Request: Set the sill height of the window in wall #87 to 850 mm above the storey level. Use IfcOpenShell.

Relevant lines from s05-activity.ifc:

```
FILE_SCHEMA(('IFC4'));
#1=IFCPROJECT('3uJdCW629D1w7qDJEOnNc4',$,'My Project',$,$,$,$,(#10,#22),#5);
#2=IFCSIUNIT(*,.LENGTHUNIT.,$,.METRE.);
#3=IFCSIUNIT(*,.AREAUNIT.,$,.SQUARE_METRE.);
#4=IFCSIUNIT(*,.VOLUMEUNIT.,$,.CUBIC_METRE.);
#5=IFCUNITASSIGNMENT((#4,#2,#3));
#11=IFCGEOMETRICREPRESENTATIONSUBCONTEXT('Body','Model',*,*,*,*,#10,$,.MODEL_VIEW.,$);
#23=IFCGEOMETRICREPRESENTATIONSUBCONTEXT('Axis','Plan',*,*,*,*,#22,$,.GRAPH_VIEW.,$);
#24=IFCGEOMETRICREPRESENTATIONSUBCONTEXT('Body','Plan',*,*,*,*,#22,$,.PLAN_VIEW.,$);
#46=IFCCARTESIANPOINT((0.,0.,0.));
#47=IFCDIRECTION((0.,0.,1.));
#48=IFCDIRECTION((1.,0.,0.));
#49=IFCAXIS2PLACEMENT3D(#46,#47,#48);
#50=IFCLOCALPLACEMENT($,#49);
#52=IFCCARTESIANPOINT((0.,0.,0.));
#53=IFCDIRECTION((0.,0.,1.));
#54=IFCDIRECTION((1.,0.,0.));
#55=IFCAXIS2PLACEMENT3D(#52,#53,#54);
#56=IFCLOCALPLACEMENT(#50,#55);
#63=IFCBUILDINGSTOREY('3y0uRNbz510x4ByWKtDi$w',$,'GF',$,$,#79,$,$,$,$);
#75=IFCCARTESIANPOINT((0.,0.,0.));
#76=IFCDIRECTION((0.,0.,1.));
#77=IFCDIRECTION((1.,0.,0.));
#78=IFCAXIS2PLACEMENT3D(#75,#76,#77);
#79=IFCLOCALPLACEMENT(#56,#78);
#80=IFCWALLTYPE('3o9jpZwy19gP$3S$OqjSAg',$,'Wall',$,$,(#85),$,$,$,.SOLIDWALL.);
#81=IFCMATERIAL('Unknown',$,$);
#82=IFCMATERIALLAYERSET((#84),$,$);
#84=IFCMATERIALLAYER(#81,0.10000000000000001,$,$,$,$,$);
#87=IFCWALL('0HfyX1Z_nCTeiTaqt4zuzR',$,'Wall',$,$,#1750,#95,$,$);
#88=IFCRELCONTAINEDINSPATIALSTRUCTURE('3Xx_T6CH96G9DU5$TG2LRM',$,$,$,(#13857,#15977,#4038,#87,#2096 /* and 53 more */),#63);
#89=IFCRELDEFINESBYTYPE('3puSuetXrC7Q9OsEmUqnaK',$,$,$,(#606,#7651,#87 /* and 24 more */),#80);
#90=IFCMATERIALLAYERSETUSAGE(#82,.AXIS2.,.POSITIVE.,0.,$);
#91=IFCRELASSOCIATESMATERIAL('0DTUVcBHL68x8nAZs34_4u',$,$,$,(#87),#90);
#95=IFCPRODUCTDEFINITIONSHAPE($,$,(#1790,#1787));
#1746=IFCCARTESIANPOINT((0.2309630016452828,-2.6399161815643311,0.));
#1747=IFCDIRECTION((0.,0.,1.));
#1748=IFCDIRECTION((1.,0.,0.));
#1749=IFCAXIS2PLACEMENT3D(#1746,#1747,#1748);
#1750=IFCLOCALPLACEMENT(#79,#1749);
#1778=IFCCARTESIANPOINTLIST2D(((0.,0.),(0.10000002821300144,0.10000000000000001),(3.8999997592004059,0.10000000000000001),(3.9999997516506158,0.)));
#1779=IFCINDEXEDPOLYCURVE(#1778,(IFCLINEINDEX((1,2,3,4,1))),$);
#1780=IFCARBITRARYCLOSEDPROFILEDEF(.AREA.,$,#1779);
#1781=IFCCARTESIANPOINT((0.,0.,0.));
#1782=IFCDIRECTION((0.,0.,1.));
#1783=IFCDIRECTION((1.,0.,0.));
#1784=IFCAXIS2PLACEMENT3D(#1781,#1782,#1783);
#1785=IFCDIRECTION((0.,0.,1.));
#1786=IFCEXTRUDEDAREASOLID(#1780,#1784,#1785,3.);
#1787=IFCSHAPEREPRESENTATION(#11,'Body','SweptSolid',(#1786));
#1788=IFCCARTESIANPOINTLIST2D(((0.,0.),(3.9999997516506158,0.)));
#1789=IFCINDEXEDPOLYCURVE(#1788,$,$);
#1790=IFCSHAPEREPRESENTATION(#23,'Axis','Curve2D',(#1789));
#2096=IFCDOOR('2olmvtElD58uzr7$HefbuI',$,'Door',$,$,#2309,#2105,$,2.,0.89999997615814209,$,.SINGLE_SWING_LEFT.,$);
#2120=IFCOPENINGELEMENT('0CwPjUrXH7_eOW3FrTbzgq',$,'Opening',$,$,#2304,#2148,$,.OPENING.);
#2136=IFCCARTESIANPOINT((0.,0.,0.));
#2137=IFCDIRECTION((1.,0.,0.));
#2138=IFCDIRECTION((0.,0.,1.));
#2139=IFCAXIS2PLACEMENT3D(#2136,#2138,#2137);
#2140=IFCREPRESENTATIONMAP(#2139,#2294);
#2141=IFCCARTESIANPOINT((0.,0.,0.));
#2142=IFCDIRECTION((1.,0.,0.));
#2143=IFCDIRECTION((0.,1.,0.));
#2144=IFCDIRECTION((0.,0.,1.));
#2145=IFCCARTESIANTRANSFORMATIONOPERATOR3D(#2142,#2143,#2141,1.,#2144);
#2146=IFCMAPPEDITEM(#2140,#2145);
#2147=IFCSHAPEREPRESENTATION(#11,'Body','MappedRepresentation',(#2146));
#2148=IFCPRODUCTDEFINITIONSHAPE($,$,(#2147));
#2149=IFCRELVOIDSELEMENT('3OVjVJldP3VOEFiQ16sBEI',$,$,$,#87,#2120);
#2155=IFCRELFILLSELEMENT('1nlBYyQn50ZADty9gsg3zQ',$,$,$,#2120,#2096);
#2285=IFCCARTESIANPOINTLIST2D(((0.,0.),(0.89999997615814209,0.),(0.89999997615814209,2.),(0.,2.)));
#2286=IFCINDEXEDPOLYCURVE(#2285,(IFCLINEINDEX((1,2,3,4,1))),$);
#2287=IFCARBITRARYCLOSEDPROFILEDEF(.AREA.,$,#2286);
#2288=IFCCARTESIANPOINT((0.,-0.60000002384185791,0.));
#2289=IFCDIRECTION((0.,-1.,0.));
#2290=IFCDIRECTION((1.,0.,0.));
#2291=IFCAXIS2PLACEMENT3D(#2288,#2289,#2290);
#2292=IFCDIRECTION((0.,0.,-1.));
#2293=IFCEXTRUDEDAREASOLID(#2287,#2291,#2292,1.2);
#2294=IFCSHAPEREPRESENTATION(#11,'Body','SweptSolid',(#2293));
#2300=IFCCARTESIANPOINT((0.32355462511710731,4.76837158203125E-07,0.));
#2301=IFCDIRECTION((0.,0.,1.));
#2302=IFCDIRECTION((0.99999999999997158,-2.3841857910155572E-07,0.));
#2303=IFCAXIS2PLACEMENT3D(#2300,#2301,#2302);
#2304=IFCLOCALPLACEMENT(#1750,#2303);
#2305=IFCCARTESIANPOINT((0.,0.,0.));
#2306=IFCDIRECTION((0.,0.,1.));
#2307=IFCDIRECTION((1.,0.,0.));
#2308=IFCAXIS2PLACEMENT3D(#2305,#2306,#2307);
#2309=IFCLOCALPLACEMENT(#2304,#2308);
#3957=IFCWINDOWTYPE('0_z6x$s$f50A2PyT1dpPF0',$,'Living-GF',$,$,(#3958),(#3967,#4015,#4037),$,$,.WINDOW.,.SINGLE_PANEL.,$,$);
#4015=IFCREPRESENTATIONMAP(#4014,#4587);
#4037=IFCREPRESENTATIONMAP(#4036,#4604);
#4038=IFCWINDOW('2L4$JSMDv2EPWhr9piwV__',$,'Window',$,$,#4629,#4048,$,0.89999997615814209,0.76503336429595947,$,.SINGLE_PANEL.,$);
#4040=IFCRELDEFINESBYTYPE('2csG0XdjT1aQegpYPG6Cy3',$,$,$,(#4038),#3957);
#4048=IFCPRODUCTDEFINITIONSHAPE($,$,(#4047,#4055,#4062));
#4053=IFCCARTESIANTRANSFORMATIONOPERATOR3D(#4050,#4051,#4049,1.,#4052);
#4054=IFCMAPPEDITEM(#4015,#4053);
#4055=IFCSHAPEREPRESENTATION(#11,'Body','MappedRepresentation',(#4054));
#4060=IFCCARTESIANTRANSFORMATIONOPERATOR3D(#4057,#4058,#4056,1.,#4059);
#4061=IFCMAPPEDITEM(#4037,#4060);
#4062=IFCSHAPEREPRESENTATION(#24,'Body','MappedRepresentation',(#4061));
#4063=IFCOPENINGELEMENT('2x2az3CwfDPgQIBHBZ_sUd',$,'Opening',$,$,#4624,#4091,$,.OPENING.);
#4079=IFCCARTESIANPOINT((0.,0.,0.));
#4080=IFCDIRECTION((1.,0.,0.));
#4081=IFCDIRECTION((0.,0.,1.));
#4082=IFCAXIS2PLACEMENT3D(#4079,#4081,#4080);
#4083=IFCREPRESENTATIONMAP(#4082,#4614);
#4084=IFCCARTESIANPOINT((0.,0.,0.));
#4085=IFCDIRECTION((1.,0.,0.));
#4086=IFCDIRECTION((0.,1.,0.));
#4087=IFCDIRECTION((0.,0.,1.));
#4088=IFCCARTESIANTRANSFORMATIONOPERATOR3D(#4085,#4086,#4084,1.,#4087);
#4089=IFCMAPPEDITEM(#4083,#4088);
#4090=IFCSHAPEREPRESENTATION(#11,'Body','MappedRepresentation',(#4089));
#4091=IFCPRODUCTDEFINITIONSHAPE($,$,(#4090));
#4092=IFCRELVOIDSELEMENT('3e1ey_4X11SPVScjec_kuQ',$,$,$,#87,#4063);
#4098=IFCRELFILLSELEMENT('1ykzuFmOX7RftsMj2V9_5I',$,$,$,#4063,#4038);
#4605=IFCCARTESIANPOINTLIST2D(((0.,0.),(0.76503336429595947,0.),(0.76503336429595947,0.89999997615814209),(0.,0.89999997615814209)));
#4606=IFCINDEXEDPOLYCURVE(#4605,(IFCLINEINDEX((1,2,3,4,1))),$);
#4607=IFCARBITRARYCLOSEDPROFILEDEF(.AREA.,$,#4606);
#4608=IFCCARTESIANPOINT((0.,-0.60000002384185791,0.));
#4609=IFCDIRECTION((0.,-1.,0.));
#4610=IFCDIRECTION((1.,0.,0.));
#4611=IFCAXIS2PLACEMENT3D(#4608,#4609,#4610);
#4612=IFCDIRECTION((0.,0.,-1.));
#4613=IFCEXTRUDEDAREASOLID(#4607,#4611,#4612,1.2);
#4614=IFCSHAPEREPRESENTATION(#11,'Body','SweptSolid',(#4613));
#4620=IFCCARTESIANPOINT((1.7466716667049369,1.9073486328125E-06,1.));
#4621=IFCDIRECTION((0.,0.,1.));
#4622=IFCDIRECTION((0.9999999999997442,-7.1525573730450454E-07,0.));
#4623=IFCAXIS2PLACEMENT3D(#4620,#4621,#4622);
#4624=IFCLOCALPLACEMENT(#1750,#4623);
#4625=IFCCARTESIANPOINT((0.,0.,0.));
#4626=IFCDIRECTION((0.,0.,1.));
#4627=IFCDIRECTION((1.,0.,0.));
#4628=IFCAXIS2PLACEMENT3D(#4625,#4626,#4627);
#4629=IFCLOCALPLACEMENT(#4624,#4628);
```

```python
import numpy as np
import ifcopenshell
import ifcopenshell.api.geometry
import ifcopenshell.geom
import ifcopenshell.util.element
import ifcopenshell.util.placement
import ifcopenshell.util.shape
import ifcopenshell.util.unit

model = ifcopenshell.open("s05-activity.ifc")
unit_scale = ifcopenshell.util.unit.calculate_unit_scale(model)

window = model.by_guid("2L4$JSMDv2EPWhr9piwV__")
opening = window.FillsVoids[0].RelatingOpeningElement
storey = ifcopenshell.util.element.get_container(window, ifc_class="IfcBuildingStorey")
level = ifcopenshell.util.placement.get_local_placement(storey.ObjectPlacement)[2, 3]

# The opening's origin need not be at the sill, so measure its lowest point.
shape = ifcopenshell.geom.create_shape(ifcopenshell.geom.settings(), opening)
bottom = ifcopenshell.util.shape.get_shape_bottom_elevation(shape, shape.geometry) / unit_scale
dz = level + 0.85 / unit_scale - bottom

shift = np.array([0.0, 0.0, dz])
# The window is placed relative to its opening, so it follows when the opening moves.
matrix = ifcopenshell.util.placement.get_local_placement(opening.ObjectPlacement)
matrix[:3, 3] += shift
ifcopenshell.api.geometry.edit_object_placement(
    model, product=opening, matrix=matrix, is_si=False, should_transform_children=True
)

print(f"moved by {dz * unit_scale:+.3f} m")

model.write("s05-activity_rev.ifc")
```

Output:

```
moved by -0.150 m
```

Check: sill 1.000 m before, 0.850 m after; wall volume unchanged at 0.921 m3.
